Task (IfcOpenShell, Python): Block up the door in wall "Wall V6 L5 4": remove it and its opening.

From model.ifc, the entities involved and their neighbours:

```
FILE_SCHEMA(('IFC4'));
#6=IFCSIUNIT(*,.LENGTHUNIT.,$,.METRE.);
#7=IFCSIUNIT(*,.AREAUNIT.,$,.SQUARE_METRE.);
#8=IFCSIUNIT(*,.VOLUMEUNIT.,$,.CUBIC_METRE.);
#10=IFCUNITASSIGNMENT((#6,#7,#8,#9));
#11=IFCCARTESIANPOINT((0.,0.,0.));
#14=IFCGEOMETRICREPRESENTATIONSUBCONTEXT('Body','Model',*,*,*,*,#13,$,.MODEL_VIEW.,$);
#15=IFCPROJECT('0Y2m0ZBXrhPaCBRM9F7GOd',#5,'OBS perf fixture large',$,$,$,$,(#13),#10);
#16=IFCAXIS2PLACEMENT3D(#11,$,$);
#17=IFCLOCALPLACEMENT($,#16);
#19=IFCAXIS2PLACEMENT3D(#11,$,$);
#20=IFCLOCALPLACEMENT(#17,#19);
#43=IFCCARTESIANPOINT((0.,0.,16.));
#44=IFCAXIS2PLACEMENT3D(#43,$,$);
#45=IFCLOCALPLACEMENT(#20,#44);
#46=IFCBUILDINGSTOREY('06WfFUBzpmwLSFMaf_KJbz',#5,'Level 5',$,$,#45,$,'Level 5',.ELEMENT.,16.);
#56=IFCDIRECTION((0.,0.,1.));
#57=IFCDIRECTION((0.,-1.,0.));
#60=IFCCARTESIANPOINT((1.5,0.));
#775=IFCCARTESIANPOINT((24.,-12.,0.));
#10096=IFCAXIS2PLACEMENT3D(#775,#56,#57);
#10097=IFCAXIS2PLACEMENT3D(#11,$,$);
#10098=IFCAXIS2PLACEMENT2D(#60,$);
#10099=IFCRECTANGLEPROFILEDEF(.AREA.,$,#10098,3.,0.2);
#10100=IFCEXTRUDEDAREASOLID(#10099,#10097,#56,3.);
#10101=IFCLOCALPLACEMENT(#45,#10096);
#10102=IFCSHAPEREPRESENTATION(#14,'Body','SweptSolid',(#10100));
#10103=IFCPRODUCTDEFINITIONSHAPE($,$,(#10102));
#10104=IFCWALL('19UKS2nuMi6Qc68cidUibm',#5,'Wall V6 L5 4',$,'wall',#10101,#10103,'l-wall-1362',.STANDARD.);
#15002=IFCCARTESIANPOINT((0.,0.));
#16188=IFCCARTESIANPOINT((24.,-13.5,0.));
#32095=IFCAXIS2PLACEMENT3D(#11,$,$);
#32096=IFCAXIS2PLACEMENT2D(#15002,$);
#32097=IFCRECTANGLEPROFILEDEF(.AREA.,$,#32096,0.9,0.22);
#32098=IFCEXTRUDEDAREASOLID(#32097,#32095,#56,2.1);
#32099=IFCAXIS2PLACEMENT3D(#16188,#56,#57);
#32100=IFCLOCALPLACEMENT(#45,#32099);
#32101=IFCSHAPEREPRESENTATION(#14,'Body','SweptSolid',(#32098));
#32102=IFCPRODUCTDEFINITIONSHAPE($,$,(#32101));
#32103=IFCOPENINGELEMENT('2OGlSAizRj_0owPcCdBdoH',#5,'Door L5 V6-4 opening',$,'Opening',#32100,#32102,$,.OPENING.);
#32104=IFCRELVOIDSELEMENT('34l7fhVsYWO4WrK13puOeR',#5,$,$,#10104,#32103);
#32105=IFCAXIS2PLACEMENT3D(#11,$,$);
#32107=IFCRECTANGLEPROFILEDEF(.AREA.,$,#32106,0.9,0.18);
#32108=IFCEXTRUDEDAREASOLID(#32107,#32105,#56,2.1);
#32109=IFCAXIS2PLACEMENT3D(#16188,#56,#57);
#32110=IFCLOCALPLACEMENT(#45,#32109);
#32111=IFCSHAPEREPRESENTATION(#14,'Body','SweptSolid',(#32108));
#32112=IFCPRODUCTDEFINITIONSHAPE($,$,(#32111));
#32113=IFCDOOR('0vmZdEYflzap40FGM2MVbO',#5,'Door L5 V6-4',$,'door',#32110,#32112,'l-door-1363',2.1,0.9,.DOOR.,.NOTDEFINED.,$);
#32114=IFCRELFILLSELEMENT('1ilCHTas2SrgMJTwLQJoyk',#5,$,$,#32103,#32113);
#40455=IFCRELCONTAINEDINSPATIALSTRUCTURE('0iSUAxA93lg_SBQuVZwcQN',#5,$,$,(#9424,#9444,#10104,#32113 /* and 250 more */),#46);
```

```python
import ifcopenshell
import ifcopenshell.api.feature
import ifcopenshell.api.root
import ifcopenshell.geom
import ifcopenshell.util.shape

model = ifcopenshell.open("model.ifc")
settings = ifcopenshell.geom.settings()


def volume(element):
    """Net volume in cubic metres, openings subtracted."""
    shape = ifcopenshell.geom.create_shape(settings, element)
    return ifcopenshell.util.shape.get_volume(shape.geometry)


door = model.by_guid("0vmZdEYflzap40FGM2MVbO")
opening = door.FillsVoids[0].RelatingOpeningElement
wall = opening.VoidsElements[0].RelatingBuildingElement
before = volume(wall)

ifcopenshell.api.root.remove_product(model, product=door)
ifcopenshell.api.feature.remove_feature(model, feature=opening)

after = volume(wall)

print(f"wall volume {before:.3f} -> {after:.3f} m3")

model.write("model_edited.ifc")
```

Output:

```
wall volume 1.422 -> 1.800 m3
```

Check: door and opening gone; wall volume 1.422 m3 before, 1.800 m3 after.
